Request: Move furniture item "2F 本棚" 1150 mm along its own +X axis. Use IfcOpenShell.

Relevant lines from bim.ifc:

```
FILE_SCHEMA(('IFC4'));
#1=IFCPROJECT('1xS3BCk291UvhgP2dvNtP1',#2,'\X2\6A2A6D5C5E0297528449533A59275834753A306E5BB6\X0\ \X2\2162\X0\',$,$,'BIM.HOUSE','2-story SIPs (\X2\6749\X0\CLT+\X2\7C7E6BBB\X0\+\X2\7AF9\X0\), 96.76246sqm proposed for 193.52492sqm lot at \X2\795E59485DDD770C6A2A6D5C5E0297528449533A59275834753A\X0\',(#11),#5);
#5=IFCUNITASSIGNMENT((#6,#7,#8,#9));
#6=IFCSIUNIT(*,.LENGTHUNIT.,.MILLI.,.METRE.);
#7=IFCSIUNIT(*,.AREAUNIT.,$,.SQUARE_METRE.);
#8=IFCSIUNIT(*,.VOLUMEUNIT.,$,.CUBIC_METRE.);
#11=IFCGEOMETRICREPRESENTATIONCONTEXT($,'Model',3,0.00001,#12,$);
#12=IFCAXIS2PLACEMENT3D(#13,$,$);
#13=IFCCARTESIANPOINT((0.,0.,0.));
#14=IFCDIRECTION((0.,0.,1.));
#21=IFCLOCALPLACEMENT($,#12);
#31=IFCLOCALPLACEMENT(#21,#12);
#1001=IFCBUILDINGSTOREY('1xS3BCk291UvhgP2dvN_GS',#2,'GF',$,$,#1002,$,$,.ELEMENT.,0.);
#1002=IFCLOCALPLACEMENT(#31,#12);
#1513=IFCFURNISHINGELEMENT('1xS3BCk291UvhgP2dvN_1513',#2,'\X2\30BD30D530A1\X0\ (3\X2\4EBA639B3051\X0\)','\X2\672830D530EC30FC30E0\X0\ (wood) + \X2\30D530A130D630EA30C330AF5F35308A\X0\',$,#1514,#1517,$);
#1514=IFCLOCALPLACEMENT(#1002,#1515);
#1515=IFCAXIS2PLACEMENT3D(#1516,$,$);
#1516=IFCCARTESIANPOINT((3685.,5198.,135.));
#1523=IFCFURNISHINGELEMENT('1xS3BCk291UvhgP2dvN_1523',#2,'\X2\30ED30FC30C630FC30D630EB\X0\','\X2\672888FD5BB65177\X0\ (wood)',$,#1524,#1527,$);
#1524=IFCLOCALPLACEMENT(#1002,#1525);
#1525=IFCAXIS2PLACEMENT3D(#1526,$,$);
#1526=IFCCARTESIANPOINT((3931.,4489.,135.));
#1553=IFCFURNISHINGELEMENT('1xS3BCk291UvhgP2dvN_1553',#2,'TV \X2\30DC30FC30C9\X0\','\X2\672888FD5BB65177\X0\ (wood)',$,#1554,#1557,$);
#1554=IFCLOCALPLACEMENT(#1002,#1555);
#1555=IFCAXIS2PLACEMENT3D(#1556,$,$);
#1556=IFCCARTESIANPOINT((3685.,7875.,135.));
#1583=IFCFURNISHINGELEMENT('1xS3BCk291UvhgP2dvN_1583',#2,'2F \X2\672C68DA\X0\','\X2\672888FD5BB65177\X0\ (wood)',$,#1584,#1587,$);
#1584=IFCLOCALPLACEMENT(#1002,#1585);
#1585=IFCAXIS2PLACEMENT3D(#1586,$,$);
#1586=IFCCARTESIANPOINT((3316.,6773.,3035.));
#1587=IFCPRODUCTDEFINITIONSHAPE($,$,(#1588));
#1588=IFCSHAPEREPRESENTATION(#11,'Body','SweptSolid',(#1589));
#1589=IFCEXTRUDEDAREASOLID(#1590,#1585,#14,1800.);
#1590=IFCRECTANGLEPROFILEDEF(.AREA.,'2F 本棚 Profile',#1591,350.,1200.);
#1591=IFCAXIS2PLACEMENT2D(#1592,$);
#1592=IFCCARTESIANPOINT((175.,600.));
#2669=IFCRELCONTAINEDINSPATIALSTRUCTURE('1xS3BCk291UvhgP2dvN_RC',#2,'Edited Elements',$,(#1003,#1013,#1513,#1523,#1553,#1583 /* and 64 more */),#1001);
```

```python
import ifcopenshell
import ifcopenshell.api.geometry
import ifcopenshell.util.placement

model = ifcopenshell.open("bim.ifc")

item = model.by_guid("1xS3BCk291UvhgP2dvN_1583")
matrix = ifcopenshell.util.placement.get_local_placement(item.ObjectPlacement)
matrix[:3, 3] += matrix[:3, 0] * 1150.0
ifcopenshell.api.geometry.edit_object_placement(model, product=item, matrix=matrix, is_si=False)

print(ifcopenshell.util.placement.get_local_placement(item.ObjectPlacement).round(3) + 0.0)

model.write("bim_rev.ifc")
```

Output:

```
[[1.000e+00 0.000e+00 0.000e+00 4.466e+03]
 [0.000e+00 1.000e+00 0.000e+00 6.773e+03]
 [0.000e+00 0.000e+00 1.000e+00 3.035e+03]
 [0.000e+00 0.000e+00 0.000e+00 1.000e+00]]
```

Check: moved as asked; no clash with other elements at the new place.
